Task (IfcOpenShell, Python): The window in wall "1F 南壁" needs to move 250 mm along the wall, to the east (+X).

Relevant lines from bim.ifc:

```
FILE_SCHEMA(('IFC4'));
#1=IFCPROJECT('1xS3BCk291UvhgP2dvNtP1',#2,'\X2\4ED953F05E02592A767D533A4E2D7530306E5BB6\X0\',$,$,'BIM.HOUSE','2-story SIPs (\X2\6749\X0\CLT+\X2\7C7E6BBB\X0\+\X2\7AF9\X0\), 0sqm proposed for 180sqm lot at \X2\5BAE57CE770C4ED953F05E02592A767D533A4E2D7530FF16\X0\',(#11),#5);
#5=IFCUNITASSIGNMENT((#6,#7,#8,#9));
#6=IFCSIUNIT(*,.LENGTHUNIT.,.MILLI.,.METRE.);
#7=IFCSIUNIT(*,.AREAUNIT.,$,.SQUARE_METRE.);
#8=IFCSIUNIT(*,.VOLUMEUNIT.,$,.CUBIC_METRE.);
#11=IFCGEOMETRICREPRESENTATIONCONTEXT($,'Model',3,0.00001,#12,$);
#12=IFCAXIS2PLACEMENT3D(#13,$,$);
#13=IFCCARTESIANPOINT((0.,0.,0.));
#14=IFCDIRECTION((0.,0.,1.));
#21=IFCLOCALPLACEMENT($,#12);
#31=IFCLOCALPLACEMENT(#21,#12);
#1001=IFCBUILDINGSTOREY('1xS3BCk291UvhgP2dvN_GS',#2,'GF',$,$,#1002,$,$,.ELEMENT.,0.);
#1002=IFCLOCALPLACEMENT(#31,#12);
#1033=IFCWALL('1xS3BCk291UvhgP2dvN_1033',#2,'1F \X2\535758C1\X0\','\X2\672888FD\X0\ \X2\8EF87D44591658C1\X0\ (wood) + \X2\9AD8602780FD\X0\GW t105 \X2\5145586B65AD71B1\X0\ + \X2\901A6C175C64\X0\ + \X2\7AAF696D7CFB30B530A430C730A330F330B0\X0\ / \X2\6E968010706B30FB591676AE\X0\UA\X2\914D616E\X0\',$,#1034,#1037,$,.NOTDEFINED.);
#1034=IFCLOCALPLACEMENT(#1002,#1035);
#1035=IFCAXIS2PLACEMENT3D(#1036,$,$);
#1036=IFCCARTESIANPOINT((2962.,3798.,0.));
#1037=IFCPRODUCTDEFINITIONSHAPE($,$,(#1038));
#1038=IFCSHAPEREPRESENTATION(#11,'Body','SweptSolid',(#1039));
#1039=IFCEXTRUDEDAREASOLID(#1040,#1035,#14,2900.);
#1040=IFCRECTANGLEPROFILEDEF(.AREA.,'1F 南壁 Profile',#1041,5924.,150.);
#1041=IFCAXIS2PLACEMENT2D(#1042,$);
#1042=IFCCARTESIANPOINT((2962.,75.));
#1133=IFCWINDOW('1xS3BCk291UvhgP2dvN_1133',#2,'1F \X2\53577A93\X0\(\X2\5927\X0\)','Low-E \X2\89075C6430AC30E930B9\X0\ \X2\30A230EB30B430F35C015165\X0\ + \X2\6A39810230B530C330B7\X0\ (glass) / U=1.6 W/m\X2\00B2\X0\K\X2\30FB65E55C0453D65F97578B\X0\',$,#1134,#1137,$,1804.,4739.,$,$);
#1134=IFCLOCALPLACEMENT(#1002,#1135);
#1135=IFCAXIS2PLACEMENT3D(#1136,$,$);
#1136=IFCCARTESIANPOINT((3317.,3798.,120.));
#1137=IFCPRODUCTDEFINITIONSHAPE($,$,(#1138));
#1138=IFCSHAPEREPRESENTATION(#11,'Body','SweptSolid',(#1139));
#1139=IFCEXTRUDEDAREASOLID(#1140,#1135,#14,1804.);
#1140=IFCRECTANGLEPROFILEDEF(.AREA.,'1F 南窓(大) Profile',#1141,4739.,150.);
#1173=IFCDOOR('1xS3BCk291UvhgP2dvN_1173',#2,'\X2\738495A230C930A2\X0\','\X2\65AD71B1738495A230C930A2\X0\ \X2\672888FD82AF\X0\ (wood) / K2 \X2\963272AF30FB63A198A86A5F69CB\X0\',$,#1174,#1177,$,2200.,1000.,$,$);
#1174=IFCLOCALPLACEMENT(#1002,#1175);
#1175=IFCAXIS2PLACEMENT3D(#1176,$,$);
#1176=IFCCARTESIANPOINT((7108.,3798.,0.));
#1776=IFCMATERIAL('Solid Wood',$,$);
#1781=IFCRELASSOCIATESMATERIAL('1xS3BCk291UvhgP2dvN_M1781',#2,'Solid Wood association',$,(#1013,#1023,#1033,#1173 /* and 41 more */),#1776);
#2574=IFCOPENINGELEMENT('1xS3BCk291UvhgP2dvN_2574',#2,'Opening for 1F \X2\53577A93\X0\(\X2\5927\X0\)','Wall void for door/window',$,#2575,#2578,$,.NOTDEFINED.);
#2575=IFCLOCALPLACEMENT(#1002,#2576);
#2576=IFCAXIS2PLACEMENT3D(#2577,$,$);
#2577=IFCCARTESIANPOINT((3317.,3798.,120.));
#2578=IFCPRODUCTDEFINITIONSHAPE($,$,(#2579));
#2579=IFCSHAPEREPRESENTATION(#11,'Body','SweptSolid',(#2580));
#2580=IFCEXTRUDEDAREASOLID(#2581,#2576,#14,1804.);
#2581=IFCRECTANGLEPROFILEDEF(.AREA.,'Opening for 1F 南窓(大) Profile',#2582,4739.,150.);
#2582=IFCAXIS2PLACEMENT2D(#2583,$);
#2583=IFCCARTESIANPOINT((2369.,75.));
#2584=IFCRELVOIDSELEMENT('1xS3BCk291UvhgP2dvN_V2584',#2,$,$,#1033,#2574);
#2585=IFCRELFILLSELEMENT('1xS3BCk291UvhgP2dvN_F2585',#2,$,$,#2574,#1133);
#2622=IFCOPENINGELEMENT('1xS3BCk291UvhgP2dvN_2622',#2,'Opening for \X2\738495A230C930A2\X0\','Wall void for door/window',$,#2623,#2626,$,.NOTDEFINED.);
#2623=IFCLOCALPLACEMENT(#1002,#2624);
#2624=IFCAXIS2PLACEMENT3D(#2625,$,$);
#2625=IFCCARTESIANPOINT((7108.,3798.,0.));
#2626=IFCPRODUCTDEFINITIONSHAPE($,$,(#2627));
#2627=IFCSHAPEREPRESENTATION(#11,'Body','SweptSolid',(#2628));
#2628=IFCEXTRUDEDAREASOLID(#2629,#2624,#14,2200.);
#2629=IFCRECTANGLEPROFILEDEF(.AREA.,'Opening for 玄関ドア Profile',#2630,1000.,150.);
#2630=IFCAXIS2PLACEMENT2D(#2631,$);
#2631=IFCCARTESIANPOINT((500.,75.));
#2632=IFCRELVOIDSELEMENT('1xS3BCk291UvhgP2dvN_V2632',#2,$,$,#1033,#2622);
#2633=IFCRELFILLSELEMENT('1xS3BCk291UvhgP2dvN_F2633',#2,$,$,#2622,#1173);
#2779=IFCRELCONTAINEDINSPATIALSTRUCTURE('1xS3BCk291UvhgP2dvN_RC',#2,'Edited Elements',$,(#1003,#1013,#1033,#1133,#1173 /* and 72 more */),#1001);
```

```python
import ifcopenshell
import ifcopenshell.api.geometry
import ifcopenshell.util.placement

model = ifcopenshell.open("bim.ifc")

window = model.by_id(1133)
opening = window.FillsVoids[0].RelatingOpeningElement
wall = opening.VoidsElements[0].RelatingBuildingElement

wall_matrix = ifcopenshell.util.placement.get_local_placement(wall.ObjectPlacement)
shift = wall_matrix[:3, 0] * 250.0
before = ifcopenshell.util.placement.get_local_placement(window.ObjectPlacement)[:3, 3].copy()

# The window is not placed relative to its opening, so move both.
for product in (opening, window):
    matrix = ifcopenshell.util.placement.get_local_placement(product.ObjectPlacement)
    matrix[:3, 3] += shift
    ifcopenshell.api.geometry.edit_object_placement(model, product=product, matrix=matrix, is_si=False)

after = ifcopenshell.util.placement.get_local_placement(window.ObjectPlacement)[:3, 3]
print("window moved by", (after - before).round(3) + 0.0)

model.write("bim_v2.ifc")
```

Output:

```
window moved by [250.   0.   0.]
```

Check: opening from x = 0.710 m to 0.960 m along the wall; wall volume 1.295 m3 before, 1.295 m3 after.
